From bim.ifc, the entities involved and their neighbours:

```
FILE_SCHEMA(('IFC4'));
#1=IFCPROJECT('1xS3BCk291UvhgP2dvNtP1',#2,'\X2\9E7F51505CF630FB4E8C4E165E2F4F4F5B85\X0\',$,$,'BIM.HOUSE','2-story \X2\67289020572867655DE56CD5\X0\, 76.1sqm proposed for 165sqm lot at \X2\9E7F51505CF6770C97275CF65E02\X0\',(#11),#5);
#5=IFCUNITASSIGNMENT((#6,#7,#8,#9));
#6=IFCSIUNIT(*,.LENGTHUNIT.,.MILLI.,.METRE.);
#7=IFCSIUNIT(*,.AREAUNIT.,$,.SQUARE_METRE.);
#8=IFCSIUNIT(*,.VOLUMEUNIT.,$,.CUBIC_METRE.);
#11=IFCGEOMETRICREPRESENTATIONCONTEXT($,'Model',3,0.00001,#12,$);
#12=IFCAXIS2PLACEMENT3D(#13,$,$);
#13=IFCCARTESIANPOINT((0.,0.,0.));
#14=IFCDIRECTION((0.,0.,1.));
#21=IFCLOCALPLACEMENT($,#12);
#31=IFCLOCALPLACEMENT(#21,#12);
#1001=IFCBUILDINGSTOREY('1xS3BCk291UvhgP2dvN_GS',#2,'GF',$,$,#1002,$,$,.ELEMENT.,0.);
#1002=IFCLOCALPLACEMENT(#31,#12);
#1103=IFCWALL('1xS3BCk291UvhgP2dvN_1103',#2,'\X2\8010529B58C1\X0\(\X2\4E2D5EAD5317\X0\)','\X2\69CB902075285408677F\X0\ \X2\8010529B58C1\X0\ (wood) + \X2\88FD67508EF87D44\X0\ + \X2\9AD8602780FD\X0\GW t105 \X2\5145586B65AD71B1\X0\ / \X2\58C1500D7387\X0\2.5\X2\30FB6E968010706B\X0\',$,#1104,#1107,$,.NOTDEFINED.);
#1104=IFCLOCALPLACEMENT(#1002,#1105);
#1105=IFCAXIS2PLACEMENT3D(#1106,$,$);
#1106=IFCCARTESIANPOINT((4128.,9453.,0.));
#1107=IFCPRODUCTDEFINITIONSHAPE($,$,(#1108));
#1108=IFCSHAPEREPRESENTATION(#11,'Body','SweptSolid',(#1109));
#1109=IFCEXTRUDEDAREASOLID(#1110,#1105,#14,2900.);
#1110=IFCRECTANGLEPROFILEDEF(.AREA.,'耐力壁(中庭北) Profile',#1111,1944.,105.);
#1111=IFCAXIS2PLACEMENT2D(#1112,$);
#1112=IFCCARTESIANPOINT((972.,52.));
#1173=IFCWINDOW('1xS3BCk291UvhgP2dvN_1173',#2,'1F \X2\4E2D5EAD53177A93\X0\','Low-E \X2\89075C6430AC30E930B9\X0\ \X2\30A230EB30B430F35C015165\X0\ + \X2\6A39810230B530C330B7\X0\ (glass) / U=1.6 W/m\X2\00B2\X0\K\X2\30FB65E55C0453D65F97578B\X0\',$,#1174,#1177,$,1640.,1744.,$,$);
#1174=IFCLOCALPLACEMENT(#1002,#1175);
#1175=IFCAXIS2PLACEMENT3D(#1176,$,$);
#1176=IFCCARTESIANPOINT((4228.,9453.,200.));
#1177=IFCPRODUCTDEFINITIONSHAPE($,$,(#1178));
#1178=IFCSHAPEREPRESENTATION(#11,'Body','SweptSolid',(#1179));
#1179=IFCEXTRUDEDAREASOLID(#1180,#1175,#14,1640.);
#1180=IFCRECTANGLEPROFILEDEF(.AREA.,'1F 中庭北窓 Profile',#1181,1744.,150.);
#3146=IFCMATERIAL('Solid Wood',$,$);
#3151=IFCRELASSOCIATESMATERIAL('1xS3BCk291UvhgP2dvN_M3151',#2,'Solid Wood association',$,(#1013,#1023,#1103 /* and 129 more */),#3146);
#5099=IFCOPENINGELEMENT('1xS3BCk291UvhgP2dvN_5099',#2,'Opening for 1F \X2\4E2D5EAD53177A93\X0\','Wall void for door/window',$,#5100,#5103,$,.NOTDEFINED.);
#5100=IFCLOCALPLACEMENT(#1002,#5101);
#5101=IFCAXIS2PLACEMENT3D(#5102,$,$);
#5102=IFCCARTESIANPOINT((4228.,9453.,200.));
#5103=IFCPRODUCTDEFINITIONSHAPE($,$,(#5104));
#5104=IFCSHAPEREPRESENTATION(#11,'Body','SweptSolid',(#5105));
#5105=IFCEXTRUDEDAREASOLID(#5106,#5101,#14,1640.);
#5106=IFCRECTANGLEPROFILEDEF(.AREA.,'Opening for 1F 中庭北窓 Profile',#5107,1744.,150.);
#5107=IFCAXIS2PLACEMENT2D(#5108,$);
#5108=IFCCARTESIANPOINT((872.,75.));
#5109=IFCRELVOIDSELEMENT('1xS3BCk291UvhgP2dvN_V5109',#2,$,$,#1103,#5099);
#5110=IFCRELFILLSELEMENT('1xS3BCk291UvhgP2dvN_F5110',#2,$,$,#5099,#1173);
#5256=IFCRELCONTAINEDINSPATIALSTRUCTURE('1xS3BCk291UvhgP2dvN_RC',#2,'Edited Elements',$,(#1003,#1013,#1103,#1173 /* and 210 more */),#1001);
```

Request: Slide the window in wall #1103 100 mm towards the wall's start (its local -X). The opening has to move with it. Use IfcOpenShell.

```python
import ifcopenshell
import ifcopenshell.api.geometry
import ifcopenshell.util.placement

model = ifcopenshell.open("bim.ifc")

window = model.by_guid("1xS3BCk291UvhgP2dvN_1173")
opening = window.FillsVoids[0].RelatingOpeningElement
wall = opening.VoidsElements[0].RelatingBuildingElement

wall_matrix = ifcopenshell.util.placement.get_local_placement(wall.ObjectPlacement)
shift = wall_matrix[:3, 0] * -100.0
before = ifcopenshell.util.placement.get_local_placement(window.ObjectPlacement)[:3, 3].copy()

# The window is not placed relative to its opening, so move both.
for product in (opening, window):
    matrix = ifcopenshell.util.placement.get_local_placement(product.ObjectPlacement)
    matrix[:3, 3] += shift
    ifcopenshell.api.geometry.edit_object_placement(model, product=product, matrix=matrix, is_si=False)

after = ifcopenshell.util.placement.get_local_placement(window.ObjectPlacement)[:3, 3]
print("window moved by", (after - before).round(3) + 0.0)

model.write("bim_updated.ifc")
```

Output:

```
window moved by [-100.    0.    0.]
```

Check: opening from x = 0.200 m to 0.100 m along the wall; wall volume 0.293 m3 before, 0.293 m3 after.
